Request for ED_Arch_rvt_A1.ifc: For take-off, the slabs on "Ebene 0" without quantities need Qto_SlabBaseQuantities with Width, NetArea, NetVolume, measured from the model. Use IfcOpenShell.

First a look at what the model holds.

```python
import ifcopenshell
import ifcopenshell.util.element
import ifcopenshell.util.unit

model = ifcopenshell.open("ED_Arch_rvt_A1.ifc")
print(model.schema)
for unit_type in ("LENGTHUNIT", "AREAUNIT", "VOLUMEUNIT"):
    print(unit_type, ifcopenshell.util.unit.calculate_unit_scale(model, unit_type))
storey = next(s for s in model.by_type("IfcBuildingStorey") if s.Name == "Ebene 0")
slabs = [e for e in ifcopenshell.util.element.get_decomposition(storey) if e.is_a("IfcSlab")]
for e in sorted(slabs, key=lambda e: e.id()):
    print(e.id(), e.is_a(), e.Name, list(ifcopenshell.util.element.get_psets(e, qtos_only=True)), sep=" | ")
```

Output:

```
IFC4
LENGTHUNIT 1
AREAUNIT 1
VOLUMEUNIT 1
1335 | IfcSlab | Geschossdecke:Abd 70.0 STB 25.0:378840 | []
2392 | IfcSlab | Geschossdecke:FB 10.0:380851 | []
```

```python
import ifcopenshell
import ifcopenshell.api.pset
import ifcopenshell.geom
import ifcopenshell.util.element
import ifcopenshell.util.shape
import ifcopenshell.util.unit

model = ifcopenshell.open("ED_Arch_rvt_A1.ifc")
unit_scale = ifcopenshell.util.unit.calculate_unit_scale(model)
area_scale = ifcopenshell.util.unit.calculate_unit_scale(model, "AREAUNIT")
volume_scale = ifcopenshell.util.unit.calculate_unit_scale(model, "VOLUMEUNIT")
settings = ifcopenshell.geom.settings()

storey = next(s for s in model.by_type("IfcBuildingStorey") if s.Name == "Ebene 0")
slabs = [e for e in ifcopenshell.util.element.get_decomposition(storey) if e.is_a("IfcSlab")]

for e in sorted(slabs, key=lambda e: e.id()):
    if ifcopenshell.util.element.get_psets(e, qtos_only=True, should_inherit=False):
        continue
    # Geometry comes back in metres, in the element's own axes.
    shape = ifcopenshell.geom.create_shape(settings, e)
    values = {
        "Width": ifcopenshell.util.shape.get_z(shape.geometry) / unit_scale,
        "NetArea": ifcopenshell.util.shape.get_footprint_area(shape.geometry) / area_scale,
        "NetVolume": ifcopenshell.util.shape.get_volume(shape.geometry) / volume_scale,
    }
    qto = ifcopenshell.api.pset.add_qto(model, product=e, name="Qto_SlabBaseQuantities")
    ifcopenshell.api.pset.edit_qto(model, qto=qto, properties=values)
    print(e.id(), {k: round(v, 3) for k, v in values.items()})

model.write("ED_Arch_rvt_A1_edited.ifc")
```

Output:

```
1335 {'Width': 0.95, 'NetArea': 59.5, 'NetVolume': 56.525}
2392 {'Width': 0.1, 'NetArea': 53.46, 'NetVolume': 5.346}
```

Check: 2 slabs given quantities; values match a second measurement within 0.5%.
